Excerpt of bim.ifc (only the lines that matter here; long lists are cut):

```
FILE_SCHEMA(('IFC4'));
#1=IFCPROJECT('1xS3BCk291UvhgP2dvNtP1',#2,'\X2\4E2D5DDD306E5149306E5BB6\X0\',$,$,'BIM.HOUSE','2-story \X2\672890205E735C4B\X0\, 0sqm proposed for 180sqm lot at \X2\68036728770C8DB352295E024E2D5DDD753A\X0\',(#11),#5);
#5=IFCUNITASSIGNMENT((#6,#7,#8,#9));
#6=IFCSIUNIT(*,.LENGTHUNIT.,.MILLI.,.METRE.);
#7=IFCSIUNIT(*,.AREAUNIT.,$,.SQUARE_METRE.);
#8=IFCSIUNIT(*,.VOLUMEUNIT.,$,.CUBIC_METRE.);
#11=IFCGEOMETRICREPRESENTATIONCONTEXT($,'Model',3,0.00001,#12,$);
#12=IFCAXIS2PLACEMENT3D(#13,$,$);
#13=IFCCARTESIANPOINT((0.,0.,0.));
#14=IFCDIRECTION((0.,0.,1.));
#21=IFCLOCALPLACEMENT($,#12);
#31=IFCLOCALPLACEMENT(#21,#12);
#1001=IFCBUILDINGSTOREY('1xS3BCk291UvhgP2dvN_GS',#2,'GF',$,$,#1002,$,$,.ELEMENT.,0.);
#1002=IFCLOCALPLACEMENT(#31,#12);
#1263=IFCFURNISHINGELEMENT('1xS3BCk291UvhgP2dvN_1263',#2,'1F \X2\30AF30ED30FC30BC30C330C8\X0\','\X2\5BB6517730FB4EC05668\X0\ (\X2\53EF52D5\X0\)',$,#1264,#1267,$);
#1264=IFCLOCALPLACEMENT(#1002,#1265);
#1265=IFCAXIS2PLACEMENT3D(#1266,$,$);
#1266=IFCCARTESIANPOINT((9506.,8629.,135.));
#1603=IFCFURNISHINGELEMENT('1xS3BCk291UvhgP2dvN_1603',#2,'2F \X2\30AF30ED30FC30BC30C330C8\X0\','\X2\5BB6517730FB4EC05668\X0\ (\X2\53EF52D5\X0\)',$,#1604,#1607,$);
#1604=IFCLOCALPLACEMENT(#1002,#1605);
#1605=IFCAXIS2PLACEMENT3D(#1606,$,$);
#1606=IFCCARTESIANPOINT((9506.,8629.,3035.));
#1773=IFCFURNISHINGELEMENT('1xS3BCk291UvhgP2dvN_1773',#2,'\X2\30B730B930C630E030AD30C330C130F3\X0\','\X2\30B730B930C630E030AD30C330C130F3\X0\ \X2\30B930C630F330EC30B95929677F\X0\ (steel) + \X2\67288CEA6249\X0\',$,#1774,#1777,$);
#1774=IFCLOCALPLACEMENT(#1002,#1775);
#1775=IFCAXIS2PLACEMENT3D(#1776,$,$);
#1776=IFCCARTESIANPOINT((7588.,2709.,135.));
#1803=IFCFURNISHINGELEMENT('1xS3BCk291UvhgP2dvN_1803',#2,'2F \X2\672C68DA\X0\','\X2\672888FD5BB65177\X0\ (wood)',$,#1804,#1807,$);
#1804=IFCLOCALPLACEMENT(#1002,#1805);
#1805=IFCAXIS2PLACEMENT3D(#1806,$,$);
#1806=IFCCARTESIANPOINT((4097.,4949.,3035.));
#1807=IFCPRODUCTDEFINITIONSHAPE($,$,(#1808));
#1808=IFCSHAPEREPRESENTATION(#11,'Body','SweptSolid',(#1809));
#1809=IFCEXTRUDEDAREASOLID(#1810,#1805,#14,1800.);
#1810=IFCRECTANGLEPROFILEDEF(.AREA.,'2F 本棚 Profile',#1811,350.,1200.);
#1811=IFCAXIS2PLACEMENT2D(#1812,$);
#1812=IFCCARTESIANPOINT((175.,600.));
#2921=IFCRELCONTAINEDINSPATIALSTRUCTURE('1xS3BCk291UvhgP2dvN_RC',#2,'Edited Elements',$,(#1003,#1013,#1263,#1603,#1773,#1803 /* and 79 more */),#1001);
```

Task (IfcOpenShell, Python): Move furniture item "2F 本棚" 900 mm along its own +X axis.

```python
import ifcopenshell
import ifcopenshell.api.geometry
import ifcopenshell.util.placement

model = ifcopenshell.open("bim.ifc")

item = model.by_guid("1xS3BCk291UvhgP2dvN_1803")
matrix = ifcopenshell.util.placement.get_local_placement(item.ObjectPlacement)
matrix[:3, 3] += matrix[:3, 0] * 900.0
ifcopenshell.api.geometry.edit_object_placement(model, product=item, matrix=matrix, is_si=False)

print(ifcopenshell.util.placement.get_local_placement(item.ObjectPlacement).round(3) + 0.0)

model.write("bim_rev.ifc")
```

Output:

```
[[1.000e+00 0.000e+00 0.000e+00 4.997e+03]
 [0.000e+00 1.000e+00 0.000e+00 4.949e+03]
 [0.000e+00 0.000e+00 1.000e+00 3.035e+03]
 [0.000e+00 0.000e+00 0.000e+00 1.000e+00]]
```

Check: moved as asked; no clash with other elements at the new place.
